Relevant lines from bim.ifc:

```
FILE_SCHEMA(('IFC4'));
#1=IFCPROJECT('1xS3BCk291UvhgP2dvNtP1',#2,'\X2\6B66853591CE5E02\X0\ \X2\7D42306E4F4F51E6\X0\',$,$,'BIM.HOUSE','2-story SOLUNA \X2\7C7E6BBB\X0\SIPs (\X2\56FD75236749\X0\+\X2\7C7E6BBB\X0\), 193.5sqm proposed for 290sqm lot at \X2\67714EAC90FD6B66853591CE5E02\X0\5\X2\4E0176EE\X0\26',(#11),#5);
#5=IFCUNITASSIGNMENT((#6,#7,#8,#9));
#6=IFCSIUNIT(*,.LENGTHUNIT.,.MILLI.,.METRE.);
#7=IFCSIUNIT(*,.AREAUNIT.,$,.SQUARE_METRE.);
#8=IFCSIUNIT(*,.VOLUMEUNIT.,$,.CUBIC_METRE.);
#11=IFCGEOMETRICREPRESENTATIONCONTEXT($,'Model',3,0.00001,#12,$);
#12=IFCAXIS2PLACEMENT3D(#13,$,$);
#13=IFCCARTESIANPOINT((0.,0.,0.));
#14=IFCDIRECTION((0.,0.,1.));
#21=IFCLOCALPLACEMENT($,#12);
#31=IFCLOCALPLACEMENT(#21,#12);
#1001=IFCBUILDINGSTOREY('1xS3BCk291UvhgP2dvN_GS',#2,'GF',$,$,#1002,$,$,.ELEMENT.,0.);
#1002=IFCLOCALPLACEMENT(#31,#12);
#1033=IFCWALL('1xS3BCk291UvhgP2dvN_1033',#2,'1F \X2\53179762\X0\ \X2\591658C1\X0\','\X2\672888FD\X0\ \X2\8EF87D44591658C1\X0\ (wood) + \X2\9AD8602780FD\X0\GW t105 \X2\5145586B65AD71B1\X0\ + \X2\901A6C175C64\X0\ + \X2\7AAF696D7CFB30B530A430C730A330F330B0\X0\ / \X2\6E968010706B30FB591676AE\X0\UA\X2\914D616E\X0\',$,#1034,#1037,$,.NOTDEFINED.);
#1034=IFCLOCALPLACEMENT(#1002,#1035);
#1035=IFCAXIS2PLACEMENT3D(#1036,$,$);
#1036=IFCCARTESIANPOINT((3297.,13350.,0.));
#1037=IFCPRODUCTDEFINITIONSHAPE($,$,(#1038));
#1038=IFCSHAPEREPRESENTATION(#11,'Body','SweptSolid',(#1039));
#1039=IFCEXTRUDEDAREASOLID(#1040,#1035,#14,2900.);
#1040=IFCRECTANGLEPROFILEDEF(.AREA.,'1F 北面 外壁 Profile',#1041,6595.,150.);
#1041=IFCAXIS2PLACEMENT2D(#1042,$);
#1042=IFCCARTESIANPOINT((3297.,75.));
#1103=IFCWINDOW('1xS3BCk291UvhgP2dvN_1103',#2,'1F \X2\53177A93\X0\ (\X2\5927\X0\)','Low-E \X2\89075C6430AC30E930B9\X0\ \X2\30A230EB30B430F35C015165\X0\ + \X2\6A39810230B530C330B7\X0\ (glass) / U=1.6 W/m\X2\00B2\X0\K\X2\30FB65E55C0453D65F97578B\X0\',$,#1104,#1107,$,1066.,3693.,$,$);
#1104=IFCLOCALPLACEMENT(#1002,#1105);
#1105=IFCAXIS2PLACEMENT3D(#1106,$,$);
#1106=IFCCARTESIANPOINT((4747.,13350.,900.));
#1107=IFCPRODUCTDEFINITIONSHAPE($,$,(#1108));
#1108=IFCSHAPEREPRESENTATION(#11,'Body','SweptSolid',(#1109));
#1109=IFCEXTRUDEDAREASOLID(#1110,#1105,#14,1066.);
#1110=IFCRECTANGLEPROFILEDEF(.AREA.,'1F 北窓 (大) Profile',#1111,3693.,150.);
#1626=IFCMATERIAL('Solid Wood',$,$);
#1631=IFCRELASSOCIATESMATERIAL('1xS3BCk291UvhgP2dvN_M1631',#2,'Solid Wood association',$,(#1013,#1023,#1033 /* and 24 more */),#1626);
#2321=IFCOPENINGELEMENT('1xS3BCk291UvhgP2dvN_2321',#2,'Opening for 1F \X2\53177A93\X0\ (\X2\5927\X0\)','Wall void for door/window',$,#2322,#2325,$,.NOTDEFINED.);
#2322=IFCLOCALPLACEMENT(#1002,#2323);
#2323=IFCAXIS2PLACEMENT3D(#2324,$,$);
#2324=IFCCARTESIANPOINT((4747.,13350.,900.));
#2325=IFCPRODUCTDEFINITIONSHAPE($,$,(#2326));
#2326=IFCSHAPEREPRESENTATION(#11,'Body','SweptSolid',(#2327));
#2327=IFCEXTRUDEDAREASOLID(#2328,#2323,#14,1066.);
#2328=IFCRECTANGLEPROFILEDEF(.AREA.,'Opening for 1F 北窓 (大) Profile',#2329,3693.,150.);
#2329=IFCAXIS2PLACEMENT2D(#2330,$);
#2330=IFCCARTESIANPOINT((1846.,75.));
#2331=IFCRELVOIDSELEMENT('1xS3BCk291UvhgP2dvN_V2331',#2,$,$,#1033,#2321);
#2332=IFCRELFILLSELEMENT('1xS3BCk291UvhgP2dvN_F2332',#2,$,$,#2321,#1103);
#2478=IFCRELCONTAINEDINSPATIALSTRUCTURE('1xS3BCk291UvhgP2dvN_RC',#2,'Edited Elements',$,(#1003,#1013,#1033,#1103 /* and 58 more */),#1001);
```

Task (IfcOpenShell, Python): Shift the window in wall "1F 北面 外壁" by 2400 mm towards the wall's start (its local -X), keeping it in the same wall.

```python
import ifcopenshell
import ifcopenshell.api.geometry
import ifcopenshell.util.placement
import ifcopenshell.util.unit

model = ifcopenshell.open("bim.ifc")
unit_scale = ifcopenshell.util.unit.calculate_unit_scale(model)

window = model.by_id(1103)
opening = window.FillsVoids[0].RelatingOpeningElement
wall = opening.VoidsElements[0].RelatingBuildingElement

wall_matrix = ifcopenshell.util.placement.get_local_placement(wall.ObjectPlacement)
shift = wall_matrix[:3, 0] * -2.4 / unit_scale
before = ifcopenshell.util.placement.get_local_placement(window.ObjectPlacement)[:3, 3].copy()

# The window is not placed relative to its opening, so move both.
for product in (opening, window):
    matrix = ifcopenshell.util.placement.get_local_placement(product.ObjectPlacement)
    matrix[:3, 3] += shift
    ifcopenshell.api.geometry.edit_object_placement(model, product=product, matrix=matrix, is_si=False)

after = ifcopenshell.util.placement.get_local_placement(window.ObjectPlacement)[:3, 3]
print("window moved by", (after - before).round(3) + 0.0)

model.write("bim_rev.ifc")
```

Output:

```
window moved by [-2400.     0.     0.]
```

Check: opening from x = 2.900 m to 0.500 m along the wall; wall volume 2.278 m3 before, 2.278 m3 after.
